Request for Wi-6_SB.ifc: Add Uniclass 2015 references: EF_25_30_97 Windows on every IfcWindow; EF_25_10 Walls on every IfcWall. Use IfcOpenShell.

First a look at what the model holds.

```python
import ifcopenshell

model = ifcopenshell.open("Wi-6_SB.ifc")
print(model.schema)
print("classifications:", [c.Name for c in model.by_type("IfcClassification")])
for ifc_class in ("IfcDoor", "IfcRoof", "IfcStair", "IfcWall", "IfcWindow"):
    print(ifc_class, len(model.by_type(ifc_class)))
```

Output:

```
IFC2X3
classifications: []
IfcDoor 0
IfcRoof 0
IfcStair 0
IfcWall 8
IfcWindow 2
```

```python
import ifcopenshell
import ifcopenshell.api.classification

model = ifcopenshell.open("Wi-6_SB.ifc")

# IFC2X3 requires Source and Edition and has no link from the project to the system.
system = model.create_entity("IfcClassification", Source="NBS", Edition="2015", Name="Uniclass 2015")

codes = {
    "IfcWindow": ("EF_25_30_97", "Windows"),
    "IfcWall": ("EF_25_10", "Walls"),
}
for ifc_class, (code, name) in codes.items():
    products = model.by_type(ifc_class)
    ifcopenshell.api.classification.add_reference(
        model, products=products, classification=system, identification=code, name=name
    )
    print(code, len(products))

model.write("Wi-6_SB_v2.ifc")
```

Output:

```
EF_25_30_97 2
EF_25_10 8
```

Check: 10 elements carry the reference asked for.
